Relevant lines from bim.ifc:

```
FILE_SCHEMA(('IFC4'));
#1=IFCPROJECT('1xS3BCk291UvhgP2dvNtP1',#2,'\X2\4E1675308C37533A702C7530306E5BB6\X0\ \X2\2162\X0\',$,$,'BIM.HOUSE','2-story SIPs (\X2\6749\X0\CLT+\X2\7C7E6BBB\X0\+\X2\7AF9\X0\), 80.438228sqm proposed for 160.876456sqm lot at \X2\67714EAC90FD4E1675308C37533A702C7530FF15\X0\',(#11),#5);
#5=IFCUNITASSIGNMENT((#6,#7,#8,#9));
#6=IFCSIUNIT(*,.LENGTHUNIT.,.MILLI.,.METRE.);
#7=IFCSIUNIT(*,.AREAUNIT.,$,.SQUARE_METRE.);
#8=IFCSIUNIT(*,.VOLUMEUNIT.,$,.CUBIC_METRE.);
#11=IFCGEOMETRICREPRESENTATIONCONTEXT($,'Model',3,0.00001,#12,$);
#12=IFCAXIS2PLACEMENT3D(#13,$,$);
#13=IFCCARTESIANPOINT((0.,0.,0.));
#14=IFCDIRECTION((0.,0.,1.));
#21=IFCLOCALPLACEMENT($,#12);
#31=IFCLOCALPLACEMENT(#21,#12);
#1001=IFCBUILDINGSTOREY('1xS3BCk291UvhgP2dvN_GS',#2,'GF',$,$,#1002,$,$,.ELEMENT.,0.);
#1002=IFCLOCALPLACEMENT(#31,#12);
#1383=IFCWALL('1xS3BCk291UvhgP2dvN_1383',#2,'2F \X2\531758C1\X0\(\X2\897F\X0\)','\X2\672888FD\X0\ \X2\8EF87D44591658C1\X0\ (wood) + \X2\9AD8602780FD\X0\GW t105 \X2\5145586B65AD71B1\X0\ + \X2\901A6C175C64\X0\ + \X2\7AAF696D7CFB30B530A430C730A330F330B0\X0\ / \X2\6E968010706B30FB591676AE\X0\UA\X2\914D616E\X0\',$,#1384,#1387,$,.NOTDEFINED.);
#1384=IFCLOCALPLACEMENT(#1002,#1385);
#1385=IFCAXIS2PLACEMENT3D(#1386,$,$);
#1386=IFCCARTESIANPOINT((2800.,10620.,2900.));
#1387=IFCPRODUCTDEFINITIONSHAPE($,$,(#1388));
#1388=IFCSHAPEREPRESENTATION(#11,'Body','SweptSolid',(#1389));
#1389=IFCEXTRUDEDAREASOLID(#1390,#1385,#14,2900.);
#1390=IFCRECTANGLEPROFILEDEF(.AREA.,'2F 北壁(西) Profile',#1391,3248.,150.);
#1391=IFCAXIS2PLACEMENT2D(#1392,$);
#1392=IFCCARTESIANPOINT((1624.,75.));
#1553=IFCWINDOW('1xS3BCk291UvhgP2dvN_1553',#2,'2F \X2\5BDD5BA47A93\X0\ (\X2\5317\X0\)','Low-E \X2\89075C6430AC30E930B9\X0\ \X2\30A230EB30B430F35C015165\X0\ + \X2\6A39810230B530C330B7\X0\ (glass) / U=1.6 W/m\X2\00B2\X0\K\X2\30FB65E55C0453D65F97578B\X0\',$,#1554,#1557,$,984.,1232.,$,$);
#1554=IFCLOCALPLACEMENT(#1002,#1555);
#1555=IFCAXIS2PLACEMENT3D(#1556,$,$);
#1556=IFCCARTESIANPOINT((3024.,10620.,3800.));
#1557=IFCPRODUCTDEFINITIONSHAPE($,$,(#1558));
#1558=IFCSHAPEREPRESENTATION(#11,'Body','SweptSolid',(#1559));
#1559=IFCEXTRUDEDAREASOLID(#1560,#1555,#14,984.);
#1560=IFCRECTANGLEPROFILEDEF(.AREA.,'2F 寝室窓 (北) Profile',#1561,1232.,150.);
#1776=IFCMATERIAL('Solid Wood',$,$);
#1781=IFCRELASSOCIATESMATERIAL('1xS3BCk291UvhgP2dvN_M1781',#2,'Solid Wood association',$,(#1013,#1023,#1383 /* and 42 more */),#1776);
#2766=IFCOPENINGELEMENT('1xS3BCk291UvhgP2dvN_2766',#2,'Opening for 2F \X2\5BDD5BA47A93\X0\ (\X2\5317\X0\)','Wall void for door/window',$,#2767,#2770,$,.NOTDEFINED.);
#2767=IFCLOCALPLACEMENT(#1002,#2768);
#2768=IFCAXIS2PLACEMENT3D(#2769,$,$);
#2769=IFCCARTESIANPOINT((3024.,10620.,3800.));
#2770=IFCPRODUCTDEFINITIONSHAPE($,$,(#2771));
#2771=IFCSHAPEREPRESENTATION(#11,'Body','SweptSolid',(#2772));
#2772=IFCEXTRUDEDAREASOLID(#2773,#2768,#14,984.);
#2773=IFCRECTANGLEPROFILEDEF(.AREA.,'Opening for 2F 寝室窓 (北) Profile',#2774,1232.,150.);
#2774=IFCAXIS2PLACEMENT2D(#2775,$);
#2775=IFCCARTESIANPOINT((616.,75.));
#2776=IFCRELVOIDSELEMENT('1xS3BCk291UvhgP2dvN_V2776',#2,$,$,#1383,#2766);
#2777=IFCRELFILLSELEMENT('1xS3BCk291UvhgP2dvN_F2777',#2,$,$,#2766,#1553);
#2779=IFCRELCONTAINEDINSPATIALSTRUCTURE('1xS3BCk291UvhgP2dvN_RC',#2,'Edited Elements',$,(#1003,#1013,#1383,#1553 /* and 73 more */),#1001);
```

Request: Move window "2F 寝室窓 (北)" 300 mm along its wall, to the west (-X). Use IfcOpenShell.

```python
import ifcopenshell
import ifcopenshell.api.geometry
import ifcopenshell.util.placement
import ifcopenshell.util.unit

model = ifcopenshell.open("bim.ifc")
unit_scale = ifcopenshell.util.unit.calculate_unit_scale(model)

window = model.by_guid("1xS3BCk291UvhgP2dvN_1553")
opening = window.FillsVoids[0].RelatingOpeningElement
wall = opening.VoidsElements[0].RelatingBuildingElement

wall_matrix = ifcopenshell.util.placement.get_local_placement(wall.ObjectPlacement)
shift = wall_matrix[:3, 0] * -0.3 / unit_scale
before = ifcopenshell.util.placement.get_local_placement(window.ObjectPlacement)[:3, 3].copy()

# The window is not placed relative to its opening, so move both.
for product in (opening, window):
    matrix = ifcopenshell.util.placement.get_local_placement(product.ObjectPlacement)
    matrix[:3, 3] += shift
    ifcopenshell.api.geometry.edit_object_placement(model, product=product, matrix=matrix, is_si=False)

after = ifcopenshell.util.placement.get_local_placement(window.ObjectPlacement)[:3, 3]
print("window moved by", (after - before).round(3) + 0.0)

model.write("bim_updated.ifc")
```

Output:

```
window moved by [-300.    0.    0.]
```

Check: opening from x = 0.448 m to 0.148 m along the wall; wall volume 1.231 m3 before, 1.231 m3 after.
